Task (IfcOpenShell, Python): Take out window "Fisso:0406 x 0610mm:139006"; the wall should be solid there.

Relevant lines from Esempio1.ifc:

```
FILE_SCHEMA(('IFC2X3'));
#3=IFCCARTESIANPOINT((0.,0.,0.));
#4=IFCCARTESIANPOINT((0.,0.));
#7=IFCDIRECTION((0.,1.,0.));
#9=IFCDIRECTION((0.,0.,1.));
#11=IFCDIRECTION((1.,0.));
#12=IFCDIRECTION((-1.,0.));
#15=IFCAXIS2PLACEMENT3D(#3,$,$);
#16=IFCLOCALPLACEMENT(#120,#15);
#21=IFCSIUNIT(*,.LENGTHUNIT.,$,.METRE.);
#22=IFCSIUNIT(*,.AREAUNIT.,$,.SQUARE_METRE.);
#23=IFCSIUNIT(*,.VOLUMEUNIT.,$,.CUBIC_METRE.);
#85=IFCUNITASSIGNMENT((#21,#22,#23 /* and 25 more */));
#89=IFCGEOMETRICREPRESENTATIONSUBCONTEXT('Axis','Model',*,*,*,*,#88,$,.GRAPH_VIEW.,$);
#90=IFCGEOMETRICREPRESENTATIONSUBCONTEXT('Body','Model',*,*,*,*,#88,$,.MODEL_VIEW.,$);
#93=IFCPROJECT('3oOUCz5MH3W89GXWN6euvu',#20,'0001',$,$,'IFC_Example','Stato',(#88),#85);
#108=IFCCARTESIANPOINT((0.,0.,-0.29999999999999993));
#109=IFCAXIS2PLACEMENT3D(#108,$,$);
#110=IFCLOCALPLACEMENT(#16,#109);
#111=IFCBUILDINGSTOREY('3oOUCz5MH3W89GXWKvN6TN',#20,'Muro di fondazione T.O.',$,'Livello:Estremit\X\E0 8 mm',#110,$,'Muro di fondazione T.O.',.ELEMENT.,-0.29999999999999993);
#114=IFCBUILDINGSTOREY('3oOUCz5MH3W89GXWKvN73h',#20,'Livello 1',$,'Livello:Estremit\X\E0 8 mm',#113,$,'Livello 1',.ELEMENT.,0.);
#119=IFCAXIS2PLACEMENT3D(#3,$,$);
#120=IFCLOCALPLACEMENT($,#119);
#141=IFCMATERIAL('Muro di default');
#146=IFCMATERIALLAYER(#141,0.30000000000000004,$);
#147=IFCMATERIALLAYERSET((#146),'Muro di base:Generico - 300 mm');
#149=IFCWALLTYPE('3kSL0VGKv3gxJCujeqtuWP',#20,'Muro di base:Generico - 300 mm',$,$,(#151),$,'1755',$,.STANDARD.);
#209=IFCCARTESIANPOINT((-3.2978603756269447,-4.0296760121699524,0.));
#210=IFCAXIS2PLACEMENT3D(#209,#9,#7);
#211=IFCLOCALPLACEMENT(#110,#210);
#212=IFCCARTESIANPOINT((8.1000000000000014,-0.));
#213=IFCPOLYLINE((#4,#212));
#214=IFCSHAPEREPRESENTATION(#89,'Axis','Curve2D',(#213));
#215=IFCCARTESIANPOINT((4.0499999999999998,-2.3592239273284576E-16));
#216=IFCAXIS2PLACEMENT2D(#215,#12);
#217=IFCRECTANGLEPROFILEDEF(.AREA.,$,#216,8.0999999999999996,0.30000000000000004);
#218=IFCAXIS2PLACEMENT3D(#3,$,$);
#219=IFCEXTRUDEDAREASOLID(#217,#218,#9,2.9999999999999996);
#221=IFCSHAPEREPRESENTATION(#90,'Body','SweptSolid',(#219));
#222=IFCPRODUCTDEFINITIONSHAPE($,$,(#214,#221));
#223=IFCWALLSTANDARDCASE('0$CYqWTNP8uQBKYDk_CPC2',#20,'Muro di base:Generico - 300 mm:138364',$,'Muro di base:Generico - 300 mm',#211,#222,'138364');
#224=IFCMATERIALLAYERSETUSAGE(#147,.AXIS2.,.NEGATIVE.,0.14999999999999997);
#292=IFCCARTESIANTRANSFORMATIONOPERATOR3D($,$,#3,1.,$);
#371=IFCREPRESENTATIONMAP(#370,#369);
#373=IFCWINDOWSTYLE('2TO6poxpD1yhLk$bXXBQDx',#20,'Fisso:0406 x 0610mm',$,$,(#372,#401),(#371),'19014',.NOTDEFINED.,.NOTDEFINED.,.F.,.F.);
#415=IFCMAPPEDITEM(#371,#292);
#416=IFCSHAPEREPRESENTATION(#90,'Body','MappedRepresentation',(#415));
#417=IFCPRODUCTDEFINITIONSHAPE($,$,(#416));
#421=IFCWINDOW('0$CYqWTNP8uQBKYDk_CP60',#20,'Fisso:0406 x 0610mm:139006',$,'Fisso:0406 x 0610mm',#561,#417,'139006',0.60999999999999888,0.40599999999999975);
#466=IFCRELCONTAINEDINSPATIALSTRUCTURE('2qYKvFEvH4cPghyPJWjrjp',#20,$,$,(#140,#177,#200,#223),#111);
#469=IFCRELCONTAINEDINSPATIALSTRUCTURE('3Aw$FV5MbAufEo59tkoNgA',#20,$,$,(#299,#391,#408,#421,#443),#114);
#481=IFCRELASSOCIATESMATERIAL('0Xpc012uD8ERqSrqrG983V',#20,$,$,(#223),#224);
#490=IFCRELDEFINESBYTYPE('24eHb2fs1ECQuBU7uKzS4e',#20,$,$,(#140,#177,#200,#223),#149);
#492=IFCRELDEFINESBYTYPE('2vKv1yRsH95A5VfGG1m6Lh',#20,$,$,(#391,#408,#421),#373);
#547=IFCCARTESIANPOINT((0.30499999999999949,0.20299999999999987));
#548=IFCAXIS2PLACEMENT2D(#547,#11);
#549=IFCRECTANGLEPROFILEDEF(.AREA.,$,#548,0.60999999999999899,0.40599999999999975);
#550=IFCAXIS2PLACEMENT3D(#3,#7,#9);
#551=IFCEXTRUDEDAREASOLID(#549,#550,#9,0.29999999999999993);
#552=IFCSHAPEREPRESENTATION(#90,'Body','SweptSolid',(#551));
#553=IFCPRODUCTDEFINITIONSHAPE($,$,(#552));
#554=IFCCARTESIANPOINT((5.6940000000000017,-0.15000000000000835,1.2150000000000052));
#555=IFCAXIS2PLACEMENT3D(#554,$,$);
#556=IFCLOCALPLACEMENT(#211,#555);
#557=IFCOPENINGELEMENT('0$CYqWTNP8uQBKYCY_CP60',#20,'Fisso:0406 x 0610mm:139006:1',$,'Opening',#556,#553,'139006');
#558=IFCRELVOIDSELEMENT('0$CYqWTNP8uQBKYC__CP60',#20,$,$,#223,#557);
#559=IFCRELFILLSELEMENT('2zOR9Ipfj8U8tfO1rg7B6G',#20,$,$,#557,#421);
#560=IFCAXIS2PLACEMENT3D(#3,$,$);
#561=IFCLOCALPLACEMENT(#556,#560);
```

```python
import ifcopenshell
import ifcopenshell.api.feature
import ifcopenshell.api.root
import ifcopenshell.geom
import ifcopenshell.util.shape

model = ifcopenshell.open("Esempio1.ifc")
settings = ifcopenshell.geom.settings()


def volume(element):
    """Net volume in cubic metres, openings subtracted."""
    shape = ifcopenshell.geom.create_shape(settings, element)
    return ifcopenshell.util.shape.get_volume(shape.geometry)


window = model.by_id(421)
opening = window.FillsVoids[0].RelatingOpeningElement
wall = opening.VoidsElements[0].RelatingBuildingElement
before = volume(wall)

ifcopenshell.api.root.remove_product(model, product=window)
ifcopenshell.api.feature.remove_feature(model, feature=opening)

after = volume(wall)

print(f"wall volume {before:.3f} -> {after:.3f} m3")

model.write("Esempio1_updated.ifc")
```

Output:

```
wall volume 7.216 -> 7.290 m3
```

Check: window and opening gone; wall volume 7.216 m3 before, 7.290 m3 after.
